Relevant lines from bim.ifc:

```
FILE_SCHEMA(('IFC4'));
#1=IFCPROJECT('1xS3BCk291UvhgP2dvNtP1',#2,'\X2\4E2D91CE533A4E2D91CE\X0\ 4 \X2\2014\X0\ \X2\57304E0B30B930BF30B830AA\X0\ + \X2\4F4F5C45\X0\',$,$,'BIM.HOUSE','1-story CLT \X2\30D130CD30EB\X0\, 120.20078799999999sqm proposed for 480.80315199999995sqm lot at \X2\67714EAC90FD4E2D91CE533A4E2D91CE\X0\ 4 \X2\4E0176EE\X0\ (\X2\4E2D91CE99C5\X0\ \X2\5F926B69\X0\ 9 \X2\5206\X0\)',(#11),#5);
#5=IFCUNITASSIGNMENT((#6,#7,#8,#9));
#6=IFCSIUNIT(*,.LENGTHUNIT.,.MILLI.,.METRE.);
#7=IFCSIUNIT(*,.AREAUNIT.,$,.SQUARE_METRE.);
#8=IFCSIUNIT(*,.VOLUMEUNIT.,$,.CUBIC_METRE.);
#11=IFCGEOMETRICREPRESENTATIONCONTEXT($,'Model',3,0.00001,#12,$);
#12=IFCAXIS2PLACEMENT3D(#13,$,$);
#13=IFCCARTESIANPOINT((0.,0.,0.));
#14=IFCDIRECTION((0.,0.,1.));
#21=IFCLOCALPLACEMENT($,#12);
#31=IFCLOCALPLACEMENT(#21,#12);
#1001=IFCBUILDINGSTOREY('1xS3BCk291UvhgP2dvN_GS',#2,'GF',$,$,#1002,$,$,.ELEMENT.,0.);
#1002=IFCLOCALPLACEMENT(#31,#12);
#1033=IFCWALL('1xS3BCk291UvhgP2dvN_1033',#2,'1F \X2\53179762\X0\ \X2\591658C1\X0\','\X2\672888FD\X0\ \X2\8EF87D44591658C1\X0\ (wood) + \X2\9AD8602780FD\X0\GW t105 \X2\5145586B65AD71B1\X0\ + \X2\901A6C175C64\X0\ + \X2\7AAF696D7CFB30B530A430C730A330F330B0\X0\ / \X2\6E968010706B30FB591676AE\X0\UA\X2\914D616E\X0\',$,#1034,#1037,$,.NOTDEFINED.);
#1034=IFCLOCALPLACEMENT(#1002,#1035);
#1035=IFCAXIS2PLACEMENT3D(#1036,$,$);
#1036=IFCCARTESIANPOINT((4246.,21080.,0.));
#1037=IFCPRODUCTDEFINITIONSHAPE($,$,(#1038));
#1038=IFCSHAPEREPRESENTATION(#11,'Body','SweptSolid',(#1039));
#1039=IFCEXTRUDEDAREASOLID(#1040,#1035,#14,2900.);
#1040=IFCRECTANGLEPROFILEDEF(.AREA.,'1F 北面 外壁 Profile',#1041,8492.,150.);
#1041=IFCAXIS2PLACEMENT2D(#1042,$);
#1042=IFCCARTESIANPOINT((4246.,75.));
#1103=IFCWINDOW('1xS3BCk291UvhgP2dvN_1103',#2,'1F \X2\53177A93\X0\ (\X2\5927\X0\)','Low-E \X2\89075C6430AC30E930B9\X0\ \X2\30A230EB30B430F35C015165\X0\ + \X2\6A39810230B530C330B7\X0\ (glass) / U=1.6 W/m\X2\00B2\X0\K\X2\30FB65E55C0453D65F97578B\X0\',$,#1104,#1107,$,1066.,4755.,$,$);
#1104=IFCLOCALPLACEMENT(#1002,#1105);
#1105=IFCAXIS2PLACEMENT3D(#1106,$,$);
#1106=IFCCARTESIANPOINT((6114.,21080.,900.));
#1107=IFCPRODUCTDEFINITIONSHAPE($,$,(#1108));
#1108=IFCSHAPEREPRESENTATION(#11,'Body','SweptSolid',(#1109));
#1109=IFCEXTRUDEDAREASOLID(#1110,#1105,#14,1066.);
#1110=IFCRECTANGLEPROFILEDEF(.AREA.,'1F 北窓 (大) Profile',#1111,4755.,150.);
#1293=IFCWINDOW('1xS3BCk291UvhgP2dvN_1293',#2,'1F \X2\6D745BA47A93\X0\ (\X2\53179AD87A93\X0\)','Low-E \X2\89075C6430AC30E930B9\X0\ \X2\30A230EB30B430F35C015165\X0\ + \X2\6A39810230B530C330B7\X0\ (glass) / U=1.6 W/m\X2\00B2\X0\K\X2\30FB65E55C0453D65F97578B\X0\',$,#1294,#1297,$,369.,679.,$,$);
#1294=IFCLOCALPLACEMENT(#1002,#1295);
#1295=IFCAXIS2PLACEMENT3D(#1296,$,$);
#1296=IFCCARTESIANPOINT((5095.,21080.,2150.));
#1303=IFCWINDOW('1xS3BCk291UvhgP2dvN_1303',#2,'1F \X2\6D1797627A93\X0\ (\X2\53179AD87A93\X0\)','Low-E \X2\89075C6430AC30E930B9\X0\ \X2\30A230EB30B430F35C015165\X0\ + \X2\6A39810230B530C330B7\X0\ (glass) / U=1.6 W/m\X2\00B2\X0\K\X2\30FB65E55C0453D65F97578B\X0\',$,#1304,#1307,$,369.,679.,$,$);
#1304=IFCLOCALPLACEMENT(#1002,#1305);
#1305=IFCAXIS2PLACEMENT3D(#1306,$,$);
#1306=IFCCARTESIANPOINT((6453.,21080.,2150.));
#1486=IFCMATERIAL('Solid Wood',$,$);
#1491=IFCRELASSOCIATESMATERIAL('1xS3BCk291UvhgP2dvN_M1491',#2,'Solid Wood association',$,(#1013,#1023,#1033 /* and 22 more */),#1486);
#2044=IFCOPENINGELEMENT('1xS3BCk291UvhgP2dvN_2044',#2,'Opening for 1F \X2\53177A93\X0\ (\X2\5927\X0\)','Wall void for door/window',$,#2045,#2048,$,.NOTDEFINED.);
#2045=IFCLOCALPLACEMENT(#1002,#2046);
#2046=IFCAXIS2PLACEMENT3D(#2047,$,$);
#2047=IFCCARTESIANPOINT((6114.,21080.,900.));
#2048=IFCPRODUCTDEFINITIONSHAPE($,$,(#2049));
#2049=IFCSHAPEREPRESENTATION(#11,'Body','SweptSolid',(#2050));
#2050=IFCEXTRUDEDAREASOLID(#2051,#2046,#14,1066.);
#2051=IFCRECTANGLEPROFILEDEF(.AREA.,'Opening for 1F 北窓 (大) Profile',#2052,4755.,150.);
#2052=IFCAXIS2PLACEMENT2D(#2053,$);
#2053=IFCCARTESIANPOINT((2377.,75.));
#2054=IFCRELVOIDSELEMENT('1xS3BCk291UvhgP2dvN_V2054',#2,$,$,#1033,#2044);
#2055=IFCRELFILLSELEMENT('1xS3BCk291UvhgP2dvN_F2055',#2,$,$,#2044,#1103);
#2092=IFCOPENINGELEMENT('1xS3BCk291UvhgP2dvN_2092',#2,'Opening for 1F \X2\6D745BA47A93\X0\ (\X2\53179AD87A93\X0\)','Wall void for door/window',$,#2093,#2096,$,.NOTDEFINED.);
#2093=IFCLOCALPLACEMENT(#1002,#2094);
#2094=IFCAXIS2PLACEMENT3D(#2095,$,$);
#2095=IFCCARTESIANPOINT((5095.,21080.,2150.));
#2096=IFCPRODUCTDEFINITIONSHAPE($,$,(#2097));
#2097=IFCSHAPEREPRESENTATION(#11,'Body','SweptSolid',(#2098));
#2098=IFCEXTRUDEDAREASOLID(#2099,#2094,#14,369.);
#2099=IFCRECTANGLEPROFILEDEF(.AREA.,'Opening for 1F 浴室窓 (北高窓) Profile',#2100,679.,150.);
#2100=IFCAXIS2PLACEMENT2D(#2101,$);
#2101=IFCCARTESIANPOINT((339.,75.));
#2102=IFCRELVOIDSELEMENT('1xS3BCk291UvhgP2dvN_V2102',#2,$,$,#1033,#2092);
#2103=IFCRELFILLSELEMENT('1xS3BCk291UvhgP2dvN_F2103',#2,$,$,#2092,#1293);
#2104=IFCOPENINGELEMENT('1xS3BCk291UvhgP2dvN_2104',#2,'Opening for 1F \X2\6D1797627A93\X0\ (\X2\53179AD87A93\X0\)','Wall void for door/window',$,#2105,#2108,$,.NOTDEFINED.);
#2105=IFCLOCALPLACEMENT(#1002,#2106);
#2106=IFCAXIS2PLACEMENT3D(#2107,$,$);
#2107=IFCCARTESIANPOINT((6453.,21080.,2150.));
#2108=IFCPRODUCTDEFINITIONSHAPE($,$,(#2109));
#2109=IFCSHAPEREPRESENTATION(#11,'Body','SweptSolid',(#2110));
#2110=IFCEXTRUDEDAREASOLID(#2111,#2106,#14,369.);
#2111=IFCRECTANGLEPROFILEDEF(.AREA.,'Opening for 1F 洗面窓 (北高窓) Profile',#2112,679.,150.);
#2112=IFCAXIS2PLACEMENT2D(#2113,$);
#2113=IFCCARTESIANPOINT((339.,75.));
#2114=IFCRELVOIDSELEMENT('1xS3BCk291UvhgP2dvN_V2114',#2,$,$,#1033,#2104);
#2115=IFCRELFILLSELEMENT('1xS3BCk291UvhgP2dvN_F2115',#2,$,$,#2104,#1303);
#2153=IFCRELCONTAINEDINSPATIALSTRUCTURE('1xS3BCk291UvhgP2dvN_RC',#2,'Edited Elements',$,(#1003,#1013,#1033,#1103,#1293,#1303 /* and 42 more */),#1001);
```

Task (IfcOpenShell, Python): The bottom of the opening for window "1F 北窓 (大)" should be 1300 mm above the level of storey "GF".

```python
import numpy as np
import ifcopenshell
import ifcopenshell.api.geometry
import ifcopenshell.geom
import ifcopenshell.util.element
import ifcopenshell.util.placement
import ifcopenshell.util.shape
import ifcopenshell.util.unit

model = ifcopenshell.open("bim.ifc")
unit_scale = ifcopenshell.util.unit.calculate_unit_scale(model)

window = model.by_guid("1xS3BCk291UvhgP2dvN_1103")
opening = window.FillsVoids[0].RelatingOpeningElement
storey = ifcopenshell.util.element.get_container(window, ifc_class="IfcBuildingStorey")
level = ifcopenshell.util.placement.get_local_placement(storey.ObjectPlacement)[2, 3]

# The opening's origin need not be at the sill, so measure its lowest point.
shape = ifcopenshell.geom.create_shape(ifcopenshell.geom.settings(), opening)
bottom = ifcopenshell.util.shape.get_shape_bottom_elevation(shape, shape.geometry) / unit_scale
dz = level + 1.3 / unit_scale - bottom

shift = np.array([0.0, 0.0, dz])
# The window is not placed relative to its opening, so move both.
for product in (opening, window):
    matrix = ifcopenshell.util.placement.get_local_placement(product.ObjectPlacement)
    matrix[:3, 3] += shift
    ifcopenshell.api.geometry.edit_object_placement(model, product=product, matrix=matrix, is_si=False)

print(f"moved by {dz * unit_scale:+.3f} m")

model.write("bim_updated.ifc")
```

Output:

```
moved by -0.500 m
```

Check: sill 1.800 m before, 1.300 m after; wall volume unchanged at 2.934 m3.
